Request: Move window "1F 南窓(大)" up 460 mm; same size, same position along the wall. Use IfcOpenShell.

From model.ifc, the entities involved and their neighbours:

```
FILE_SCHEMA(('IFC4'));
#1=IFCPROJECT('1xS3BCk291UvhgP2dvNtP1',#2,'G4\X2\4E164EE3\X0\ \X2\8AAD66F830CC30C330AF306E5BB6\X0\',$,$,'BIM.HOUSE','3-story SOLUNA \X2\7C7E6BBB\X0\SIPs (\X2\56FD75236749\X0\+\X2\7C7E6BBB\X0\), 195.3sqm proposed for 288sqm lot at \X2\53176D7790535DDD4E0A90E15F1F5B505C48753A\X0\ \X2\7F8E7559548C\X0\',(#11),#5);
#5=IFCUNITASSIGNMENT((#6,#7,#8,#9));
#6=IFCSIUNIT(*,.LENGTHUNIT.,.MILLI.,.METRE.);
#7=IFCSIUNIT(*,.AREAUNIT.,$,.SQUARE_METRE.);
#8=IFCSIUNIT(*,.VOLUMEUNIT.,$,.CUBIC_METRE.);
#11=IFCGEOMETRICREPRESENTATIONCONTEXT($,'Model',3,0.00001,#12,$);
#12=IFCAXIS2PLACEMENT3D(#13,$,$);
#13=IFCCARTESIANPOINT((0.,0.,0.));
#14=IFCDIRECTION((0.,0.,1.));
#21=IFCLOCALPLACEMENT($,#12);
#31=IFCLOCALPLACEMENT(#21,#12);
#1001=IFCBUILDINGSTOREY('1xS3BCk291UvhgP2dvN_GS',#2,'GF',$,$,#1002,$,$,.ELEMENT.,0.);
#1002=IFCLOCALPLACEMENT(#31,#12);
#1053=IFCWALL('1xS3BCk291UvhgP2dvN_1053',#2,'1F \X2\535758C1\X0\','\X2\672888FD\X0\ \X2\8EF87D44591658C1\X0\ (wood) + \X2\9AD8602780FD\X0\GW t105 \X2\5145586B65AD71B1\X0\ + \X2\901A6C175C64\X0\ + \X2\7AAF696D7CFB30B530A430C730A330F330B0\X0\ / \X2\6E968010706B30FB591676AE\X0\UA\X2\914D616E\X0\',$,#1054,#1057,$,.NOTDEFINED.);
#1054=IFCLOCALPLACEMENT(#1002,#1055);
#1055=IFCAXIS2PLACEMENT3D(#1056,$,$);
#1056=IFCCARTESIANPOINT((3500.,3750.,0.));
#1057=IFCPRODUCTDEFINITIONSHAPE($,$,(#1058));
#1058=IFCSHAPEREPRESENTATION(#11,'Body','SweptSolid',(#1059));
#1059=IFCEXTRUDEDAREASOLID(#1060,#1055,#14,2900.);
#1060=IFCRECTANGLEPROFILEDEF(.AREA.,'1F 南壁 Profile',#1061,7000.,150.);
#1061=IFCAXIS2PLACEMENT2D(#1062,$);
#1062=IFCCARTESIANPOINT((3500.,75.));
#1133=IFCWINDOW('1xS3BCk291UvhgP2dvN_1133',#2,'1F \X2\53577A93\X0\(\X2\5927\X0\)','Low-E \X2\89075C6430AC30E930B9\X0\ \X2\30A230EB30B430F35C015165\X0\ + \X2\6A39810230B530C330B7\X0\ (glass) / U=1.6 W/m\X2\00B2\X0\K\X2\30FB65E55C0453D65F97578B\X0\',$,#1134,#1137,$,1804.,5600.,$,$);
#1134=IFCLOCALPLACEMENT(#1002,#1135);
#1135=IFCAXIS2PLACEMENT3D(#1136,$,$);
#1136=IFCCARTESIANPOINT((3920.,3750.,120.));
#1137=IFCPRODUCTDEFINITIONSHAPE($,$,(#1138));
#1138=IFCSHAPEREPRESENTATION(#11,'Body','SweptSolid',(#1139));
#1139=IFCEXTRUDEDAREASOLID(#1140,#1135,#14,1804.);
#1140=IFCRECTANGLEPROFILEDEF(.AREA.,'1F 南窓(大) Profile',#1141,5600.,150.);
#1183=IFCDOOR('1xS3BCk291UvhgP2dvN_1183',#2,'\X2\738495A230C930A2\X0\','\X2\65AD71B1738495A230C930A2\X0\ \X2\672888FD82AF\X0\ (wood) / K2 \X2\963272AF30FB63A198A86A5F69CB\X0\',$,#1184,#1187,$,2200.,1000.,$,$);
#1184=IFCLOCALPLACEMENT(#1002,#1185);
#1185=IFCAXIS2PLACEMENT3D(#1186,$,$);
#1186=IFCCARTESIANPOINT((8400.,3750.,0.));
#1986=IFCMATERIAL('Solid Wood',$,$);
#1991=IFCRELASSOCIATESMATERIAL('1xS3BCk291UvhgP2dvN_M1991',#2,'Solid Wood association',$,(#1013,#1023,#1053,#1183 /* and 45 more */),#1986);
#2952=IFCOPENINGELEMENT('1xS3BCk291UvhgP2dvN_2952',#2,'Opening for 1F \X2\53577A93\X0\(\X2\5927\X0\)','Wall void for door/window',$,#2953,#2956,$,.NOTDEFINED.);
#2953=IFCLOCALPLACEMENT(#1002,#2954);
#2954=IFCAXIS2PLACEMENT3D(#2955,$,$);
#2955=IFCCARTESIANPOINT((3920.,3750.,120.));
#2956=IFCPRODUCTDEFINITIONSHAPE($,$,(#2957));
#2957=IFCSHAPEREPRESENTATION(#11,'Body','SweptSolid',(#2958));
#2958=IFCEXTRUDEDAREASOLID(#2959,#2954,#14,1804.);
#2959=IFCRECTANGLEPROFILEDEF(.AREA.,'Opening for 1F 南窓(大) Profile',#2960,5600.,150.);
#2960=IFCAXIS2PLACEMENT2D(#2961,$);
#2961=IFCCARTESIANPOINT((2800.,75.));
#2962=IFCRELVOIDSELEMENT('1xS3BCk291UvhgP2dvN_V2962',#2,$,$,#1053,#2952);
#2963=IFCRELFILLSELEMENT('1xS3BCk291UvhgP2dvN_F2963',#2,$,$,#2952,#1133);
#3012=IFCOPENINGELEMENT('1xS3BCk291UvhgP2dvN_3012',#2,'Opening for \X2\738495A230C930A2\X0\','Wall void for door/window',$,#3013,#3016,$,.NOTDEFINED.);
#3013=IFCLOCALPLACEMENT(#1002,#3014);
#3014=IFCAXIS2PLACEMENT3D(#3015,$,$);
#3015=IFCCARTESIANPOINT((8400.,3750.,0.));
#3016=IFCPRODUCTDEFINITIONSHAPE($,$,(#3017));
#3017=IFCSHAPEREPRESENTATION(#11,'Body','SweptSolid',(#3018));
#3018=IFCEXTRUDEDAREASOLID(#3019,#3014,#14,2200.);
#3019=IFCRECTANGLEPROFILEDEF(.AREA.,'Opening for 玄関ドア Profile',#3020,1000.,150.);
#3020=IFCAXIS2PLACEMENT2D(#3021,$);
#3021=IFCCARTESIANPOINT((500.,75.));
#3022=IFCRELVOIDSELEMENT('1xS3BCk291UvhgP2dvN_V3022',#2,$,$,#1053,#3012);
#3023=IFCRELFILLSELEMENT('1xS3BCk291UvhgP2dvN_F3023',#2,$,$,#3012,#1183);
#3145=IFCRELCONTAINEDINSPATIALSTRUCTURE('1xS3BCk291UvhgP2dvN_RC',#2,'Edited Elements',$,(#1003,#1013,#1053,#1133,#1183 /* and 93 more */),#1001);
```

```python
import numpy as np
import ifcopenshell
import ifcopenshell.api.geometry
import ifcopenshell.util.placement
import ifcopenshell.util.unit

model = ifcopenshell.open("model.ifc")
unit_scale = ifcopenshell.util.unit.calculate_unit_scale(model)

window = model.by_guid("1xS3BCk291UvhgP2dvN_1133")
opening = window.FillsVoids[0].RelatingOpeningElement
dz = 0.46 / unit_scale

shift = np.array([0.0, 0.0, dz])
# The window is not placed relative to its opening, so move both.
for product in (opening, window):
    matrix = ifcopenshell.util.placement.get_local_placement(product.ObjectPlacement)
    matrix[:3, 3] += shift
    ifcopenshell.api.geometry.edit_object_placement(model, product=product, matrix=matrix, is_si=False)

print(f"moved by {dz * unit_scale:+.3f} m")

model.write("model_rev.ifc")
```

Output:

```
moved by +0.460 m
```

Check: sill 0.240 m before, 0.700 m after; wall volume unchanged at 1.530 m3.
